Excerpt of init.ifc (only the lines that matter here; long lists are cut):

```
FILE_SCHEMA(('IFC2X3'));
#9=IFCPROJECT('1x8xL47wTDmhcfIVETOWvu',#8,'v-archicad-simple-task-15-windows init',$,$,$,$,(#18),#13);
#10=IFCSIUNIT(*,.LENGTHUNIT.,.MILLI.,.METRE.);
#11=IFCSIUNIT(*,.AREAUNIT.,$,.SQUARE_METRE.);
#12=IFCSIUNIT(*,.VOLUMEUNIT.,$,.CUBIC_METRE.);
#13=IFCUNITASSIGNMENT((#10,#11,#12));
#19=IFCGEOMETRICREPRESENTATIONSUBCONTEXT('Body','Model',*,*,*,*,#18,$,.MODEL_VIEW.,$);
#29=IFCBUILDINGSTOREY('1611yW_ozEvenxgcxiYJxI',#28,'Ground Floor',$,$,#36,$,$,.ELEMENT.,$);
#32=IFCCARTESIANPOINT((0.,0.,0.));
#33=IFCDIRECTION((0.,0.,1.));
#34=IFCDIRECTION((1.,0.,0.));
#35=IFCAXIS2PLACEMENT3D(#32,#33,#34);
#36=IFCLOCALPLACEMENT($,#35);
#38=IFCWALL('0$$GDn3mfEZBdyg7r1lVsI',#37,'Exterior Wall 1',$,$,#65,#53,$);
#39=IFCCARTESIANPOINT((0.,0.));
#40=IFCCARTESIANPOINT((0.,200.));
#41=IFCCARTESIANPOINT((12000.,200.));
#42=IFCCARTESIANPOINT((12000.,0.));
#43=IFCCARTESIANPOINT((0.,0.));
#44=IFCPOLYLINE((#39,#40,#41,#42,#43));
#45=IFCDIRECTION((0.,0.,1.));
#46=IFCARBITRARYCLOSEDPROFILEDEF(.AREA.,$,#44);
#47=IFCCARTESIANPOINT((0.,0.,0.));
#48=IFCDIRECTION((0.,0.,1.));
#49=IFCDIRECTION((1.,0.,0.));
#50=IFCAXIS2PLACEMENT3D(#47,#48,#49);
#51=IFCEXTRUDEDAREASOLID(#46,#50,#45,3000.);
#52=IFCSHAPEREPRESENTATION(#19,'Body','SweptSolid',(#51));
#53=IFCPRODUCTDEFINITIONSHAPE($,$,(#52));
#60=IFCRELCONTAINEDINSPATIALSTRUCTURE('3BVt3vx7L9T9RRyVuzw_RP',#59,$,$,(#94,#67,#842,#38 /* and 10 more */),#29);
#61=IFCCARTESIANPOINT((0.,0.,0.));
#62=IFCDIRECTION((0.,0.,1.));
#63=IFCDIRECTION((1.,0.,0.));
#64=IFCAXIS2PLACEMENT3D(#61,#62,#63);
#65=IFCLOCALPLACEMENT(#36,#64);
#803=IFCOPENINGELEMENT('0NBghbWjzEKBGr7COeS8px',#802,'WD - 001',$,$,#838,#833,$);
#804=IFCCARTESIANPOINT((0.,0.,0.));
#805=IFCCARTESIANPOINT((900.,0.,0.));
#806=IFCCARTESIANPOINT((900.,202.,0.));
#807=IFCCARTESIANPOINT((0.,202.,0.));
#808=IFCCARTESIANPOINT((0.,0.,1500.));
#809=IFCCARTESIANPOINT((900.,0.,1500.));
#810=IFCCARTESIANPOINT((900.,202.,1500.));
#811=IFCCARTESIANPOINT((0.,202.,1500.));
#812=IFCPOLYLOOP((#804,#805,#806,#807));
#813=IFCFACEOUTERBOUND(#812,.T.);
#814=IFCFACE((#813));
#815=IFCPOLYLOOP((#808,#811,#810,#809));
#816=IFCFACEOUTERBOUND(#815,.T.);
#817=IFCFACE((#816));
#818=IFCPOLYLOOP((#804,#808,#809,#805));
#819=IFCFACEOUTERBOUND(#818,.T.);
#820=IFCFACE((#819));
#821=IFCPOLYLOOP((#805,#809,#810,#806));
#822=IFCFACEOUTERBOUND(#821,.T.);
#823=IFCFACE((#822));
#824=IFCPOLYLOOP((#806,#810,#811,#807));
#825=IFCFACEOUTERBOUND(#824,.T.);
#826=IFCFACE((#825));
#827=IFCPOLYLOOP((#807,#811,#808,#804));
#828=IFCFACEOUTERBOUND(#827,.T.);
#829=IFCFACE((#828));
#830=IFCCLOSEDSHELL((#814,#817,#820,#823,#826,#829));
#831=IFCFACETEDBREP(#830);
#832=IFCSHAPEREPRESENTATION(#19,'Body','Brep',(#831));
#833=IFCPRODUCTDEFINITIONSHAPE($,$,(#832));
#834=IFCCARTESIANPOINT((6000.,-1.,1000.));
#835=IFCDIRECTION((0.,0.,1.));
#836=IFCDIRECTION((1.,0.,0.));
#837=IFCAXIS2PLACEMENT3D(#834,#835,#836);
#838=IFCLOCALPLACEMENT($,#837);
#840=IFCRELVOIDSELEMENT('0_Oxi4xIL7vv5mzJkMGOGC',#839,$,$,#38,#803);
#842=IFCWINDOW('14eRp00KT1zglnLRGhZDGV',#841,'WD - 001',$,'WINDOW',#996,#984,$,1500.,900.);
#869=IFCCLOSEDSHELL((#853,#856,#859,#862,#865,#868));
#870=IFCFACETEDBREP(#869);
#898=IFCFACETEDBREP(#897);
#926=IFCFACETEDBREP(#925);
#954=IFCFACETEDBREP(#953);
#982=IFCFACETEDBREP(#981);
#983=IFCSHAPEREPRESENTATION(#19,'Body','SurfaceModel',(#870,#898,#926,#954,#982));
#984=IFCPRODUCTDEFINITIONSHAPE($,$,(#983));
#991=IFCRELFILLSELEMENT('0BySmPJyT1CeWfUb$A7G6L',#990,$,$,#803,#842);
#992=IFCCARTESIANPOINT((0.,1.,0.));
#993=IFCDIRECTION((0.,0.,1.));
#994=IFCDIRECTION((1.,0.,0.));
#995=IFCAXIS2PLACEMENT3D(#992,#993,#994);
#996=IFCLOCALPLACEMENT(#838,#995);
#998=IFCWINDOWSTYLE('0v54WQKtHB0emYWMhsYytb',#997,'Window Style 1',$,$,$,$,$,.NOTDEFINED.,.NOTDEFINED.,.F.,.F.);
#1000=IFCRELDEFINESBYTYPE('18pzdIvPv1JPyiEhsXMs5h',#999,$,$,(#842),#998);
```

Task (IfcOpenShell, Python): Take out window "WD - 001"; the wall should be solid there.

```python
import ifcopenshell
import ifcopenshell.api.feature
import ifcopenshell.api.root
import ifcopenshell.geom
import ifcopenshell.util.shape

model = ifcopenshell.open("init.ifc")
settings = ifcopenshell.geom.settings()


def volume(element):
    """Net volume in cubic metres, openings subtracted."""
    shape = ifcopenshell.geom.create_shape(settings, element)
    return ifcopenshell.util.shape.get_volume(shape.geometry)


window = model.by_guid("14eRp00KT1zglnLRGhZDGV")
opening = window.FillsVoids[0].RelatingOpeningElement
wall = opening.VoidsElements[0].RelatingBuildingElement
before = volume(wall)

ifcopenshell.api.root.remove_product(model, product=window)
ifcopenshell.api.feature.remove_feature(model, feature=opening)

after = volume(wall)

print(f"wall volume {before:.3f} -> {after:.3f} m3")

model.write("init-out.ifc")
```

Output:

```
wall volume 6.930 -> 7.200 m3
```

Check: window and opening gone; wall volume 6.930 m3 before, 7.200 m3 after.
